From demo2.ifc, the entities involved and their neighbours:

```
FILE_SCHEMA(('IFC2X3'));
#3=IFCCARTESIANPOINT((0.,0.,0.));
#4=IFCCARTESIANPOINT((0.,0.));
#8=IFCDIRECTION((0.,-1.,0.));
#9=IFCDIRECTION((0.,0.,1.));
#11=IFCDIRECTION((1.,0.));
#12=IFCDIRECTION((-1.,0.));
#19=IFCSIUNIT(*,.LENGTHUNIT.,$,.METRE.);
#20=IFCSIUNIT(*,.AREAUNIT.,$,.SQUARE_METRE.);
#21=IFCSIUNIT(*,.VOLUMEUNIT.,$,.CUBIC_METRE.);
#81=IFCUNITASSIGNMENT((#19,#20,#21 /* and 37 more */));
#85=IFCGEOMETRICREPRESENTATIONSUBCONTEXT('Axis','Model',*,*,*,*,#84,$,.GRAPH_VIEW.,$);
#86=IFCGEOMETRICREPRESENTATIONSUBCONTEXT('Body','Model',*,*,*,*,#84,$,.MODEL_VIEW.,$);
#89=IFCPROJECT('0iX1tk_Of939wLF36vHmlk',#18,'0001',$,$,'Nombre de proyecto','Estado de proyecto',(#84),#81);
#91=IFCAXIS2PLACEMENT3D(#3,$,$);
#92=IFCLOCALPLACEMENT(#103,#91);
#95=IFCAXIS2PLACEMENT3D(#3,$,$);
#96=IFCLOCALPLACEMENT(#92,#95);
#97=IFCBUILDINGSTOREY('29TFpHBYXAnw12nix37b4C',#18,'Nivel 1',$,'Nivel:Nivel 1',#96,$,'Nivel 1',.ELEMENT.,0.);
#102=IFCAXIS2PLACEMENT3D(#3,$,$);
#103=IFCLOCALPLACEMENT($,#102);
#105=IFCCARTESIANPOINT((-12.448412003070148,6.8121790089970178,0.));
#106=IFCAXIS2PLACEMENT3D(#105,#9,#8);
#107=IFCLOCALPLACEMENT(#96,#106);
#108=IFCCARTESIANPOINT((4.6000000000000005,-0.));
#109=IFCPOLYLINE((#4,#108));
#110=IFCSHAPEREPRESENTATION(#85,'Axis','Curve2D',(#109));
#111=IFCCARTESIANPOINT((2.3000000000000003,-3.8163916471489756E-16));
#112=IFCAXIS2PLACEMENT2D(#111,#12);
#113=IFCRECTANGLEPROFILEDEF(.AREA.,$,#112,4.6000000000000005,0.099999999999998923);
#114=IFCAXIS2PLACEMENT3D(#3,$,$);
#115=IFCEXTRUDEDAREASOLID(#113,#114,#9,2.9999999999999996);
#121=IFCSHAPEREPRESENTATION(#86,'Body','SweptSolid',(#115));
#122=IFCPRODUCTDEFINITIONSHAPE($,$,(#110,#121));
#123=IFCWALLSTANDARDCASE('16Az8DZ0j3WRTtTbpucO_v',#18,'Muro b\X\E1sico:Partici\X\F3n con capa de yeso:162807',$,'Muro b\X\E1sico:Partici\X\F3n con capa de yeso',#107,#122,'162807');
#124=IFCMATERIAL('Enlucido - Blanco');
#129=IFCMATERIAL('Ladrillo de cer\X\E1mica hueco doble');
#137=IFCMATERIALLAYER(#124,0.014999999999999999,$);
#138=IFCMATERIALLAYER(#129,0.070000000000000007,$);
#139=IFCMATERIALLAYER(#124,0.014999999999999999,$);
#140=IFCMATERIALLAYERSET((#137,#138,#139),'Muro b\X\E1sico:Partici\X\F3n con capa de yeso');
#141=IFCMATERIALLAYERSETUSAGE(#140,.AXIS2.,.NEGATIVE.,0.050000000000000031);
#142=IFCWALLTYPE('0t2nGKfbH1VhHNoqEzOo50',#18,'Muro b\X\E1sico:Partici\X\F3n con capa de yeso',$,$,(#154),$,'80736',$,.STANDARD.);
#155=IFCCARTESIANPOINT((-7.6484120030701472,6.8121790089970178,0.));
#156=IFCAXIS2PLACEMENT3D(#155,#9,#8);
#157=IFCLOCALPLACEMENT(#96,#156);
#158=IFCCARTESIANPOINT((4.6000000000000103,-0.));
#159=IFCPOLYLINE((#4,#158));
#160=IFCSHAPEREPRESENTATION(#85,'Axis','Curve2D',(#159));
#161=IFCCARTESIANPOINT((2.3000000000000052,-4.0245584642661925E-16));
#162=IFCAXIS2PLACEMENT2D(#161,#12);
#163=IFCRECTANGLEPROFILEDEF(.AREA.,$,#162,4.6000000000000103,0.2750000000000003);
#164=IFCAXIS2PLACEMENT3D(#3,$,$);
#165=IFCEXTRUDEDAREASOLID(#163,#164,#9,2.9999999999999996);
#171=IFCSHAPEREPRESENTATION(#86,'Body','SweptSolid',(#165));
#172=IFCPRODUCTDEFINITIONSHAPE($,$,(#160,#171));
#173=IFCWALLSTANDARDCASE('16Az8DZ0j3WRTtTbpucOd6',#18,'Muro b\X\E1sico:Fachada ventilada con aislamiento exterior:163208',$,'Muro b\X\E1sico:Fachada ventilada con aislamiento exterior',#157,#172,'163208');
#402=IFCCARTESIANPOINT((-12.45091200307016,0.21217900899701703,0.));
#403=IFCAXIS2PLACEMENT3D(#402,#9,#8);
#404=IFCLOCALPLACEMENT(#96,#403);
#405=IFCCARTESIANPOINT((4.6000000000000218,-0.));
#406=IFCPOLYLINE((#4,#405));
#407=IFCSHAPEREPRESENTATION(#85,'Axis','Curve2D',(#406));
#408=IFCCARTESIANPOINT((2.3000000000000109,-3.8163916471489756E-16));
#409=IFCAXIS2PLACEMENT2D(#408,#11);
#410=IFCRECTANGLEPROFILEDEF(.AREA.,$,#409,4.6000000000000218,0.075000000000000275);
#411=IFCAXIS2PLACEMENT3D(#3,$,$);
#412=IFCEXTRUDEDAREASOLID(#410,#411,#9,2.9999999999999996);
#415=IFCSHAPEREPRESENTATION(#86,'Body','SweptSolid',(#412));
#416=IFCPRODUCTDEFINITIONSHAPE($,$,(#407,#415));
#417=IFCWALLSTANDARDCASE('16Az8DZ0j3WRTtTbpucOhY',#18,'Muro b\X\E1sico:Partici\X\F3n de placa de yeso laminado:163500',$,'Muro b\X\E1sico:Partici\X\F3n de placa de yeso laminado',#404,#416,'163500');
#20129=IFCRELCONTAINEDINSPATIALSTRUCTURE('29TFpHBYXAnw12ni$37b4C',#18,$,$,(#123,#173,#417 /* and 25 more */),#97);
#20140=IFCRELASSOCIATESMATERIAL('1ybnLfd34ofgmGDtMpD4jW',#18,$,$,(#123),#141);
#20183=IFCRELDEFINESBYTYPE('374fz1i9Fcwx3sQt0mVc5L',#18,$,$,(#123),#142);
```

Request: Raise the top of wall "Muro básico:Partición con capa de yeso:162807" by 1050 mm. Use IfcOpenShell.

```python
import ifcopenshell
import ifcopenshell.geom
import ifcopenshell.util.representation
import ifcopenshell.util.shape

model = ifcopenshell.open("demo2.ifc")
settings = ifcopenshell.geom.settings()


def volume(element):
    """Net volume in cubic metres, openings subtracted."""
    shape = ifcopenshell.geom.create_shape(settings, element)
    return ifcopenshell.util.shape.get_volume(shape.geometry)


wall = model.by_guid("16Az8DZ0j3WRTtTbpucO_v")
before = volume(wall)

body = ifcopenshell.util.representation.get_representation(wall, "Model", "Body")
solid = body.Items[0]
old_height = solid.Depth
solid.Depth += 1.05
after = volume(wall)

print(f"height {old_height:g} -> {solid.Depth:g}, volume {before:.3f} -> {after:.3f} m3")

model.write("demo2-out.ifc")
```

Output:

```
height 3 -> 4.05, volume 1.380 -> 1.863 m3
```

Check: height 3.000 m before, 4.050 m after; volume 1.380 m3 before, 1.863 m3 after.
